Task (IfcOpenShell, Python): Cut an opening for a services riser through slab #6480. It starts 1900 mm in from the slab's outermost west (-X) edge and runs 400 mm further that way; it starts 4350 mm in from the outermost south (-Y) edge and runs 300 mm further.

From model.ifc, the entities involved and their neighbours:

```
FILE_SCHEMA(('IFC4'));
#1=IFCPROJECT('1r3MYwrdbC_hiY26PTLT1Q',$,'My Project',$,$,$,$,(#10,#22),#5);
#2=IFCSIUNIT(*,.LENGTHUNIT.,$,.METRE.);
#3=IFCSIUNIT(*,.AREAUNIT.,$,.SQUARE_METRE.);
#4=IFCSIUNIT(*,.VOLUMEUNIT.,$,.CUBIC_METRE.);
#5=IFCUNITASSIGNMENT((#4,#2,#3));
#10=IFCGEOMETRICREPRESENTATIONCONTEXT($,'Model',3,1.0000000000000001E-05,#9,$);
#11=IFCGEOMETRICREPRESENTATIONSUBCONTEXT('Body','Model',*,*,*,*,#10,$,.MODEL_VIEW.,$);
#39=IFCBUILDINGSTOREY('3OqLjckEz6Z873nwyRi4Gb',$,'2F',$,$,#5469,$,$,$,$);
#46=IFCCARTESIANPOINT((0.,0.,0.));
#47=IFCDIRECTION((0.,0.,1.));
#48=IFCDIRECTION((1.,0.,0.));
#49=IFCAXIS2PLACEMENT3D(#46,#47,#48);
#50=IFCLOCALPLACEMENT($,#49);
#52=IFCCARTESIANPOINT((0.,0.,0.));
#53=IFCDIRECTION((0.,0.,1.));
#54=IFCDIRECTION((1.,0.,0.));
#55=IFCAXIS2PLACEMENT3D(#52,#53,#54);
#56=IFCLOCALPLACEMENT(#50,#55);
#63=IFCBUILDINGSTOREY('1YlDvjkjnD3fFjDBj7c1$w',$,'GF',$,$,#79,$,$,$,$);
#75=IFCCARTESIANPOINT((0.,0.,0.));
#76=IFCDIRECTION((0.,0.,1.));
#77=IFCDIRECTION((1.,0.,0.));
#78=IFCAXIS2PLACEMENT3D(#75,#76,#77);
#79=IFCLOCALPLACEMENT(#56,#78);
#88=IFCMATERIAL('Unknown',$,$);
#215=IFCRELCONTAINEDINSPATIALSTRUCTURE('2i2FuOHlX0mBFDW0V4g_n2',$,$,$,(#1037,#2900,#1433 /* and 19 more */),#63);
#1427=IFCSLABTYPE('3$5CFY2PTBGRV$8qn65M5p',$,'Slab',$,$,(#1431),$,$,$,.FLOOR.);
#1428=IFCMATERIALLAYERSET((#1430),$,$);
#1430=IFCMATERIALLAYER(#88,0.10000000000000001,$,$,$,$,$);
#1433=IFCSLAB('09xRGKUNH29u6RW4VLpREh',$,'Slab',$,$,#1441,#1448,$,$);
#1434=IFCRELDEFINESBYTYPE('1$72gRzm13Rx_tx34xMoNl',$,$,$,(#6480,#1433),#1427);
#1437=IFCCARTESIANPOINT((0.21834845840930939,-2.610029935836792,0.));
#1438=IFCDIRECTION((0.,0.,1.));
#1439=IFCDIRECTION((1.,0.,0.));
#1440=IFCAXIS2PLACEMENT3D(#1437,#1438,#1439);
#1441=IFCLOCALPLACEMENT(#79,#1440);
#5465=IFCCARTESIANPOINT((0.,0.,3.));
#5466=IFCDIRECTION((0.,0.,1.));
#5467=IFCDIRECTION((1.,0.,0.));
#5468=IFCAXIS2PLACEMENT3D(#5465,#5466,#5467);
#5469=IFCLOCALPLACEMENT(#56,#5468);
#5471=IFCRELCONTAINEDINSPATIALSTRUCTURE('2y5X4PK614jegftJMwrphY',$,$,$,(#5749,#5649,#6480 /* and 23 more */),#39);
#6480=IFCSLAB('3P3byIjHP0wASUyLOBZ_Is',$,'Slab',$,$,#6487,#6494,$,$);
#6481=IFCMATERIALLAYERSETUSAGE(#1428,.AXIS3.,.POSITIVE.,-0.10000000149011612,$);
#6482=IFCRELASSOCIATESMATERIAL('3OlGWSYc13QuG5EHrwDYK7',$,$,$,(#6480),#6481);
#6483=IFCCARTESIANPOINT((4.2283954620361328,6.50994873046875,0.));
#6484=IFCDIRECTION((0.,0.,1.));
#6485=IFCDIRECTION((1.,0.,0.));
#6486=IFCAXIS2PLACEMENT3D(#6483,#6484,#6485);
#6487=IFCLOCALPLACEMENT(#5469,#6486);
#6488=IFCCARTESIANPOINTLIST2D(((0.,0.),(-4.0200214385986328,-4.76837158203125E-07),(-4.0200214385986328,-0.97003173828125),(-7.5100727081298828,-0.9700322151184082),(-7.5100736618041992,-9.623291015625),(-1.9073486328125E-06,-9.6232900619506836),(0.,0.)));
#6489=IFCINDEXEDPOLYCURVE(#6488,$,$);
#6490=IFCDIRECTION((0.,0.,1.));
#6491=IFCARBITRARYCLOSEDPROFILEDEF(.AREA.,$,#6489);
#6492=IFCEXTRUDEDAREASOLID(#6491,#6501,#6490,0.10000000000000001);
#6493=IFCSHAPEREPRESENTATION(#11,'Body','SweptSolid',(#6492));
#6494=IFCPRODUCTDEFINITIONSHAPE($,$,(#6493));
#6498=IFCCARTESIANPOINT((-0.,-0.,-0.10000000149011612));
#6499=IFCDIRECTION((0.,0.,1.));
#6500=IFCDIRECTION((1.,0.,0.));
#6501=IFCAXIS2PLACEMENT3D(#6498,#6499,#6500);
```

```python
import numpy as np
import ifcopenshell
import ifcopenshell.api.feature
import ifcopenshell.api.geometry
import ifcopenshell.api.root
import ifcopenshell.geom
import ifcopenshell.util.placement
import ifcopenshell.util.representation
import ifcopenshell.util.shape
import ifcopenshell.util.unit

model = ifcopenshell.open("model.ifc")
unit_scale = ifcopenshell.util.unit.calculate_unit_scale(model)
settings = ifcopenshell.geom.settings()


def volume(element):
    """Net volume in cubic metres, openings subtracted."""
    shape = ifcopenshell.geom.create_shape(settings, element)
    return ifcopenshell.util.shape.get_volume(shape.geometry)


slab = model.by_guid("3P3byIjHP0wASUyLOBZ_Is")
before = volume(slab)

# Extent in the slab's own axes, in metres. The edges named are its -X and -Y sides.
slab_shape = ifcopenshell.geom.create_shape(settings, slab)
vertices = ifcopenshell.util.shape.get_vertices(slab_shape.geometry)
x_min, y_min, bottom = vertices.min(axis=0)
top = vertices[:, 2].max()

opening = ifcopenshell.api.root.create_entity(model, ifc_class="IfcOpeningElement", name="Services riser opening", predefined_type="OPENING")
context = ifcopenshell.util.representation.get_context(model, "Model", "Body", "MODEL_VIEW")
width, depth = 0.4, 0.3
outline = [(0.0, 0.0), (width, 0.0), (width, depth), (0.0, depth), (0.0, 0.0)]
# Overshoot both faces by 50 mm so the cut is clean.
shape = ifcopenshell.api.geometry.add_slab_representation(
    model, context=context, depth=top - bottom + 0.1, polyline=outline
)
ifcopenshell.api.geometry.assign_representation(model, product=opening, representation=shape)

matrix = ifcopenshell.util.placement.get_local_placement(slab.ObjectPlacement)
matrix[:, 3] = matrix @ np.append(np.array([x_min + 1.9, y_min + 4.35, bottom - 0.05]) / unit_scale, 1.0)
ifcopenshell.api.geometry.edit_object_placement(model, product=opening, matrix=matrix, is_si=False)
ifcopenshell.api.feature.add_feature(model, feature=opening, element=slab)

after = volume(slab)

print(f"slab volume {before:.3f} -> {after:.3f} m3")

model.write("model_rev.ifc")
```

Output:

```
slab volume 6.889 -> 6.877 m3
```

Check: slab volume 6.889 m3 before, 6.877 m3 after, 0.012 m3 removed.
